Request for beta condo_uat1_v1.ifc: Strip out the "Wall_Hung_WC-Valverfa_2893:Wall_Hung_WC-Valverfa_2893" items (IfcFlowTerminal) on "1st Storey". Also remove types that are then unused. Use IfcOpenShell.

First a look at what the model holds.

```python
import ifcopenshell
import ifcopenshell.util.element

model = ifcopenshell.open("beta condo_uat1_v1.ifc")
print(model.schema)
storey = next(s for s in model.by_type("IfcBuildingStorey") if s.Name == "1st Storey")
terminals = [e for e in ifcopenshell.util.element.get_decomposition(storey) if e.is_a("IfcFlowTerminal")]
seen = {}
for e in terminals:
    element_type = ifcopenshell.util.element.get_type(e)
    name = element_type.Name if element_type not in (None, e) else None
    seen[name] = seen.get(name, 0) + 1
for name, count in sorted(seen.items(), key=str):
    print(count, "x", name)
```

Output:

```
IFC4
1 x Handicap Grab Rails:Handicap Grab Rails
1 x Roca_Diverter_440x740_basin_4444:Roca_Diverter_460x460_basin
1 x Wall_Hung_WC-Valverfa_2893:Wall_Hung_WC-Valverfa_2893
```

```python
import ifcopenshell
import ifcopenshell.api.root
import ifcopenshell.util.element

model = ifcopenshell.open("beta condo_uat1_v1.ifc")

storey = next(s for s in model.by_type("IfcBuildingStorey") if s.Name == "1st Storey")
terminals = [e for e in ifcopenshell.util.element.get_decomposition(storey) if e.is_a("IfcFlowTerminal")]
targets = [e for e in terminals if (t := ifcopenshell.util.element.get_type(e)) not in (None, e) and t.Name == "Wall_Hung_WC-Valverfa_2893:Wall_Hung_WC-Valverfa_2893"]
types = {ifcopenshell.util.element.get_type(e) for e in targets} - {None, *targets}

for e in targets:
    ifcopenshell.api.root.remove_product(model, product=e)
print(len(targets), "removed")

unused = [t for t in types if not ifcopenshell.util.element.get_types(t)]
for t in unused:
    ifcopenshell.api.root.remove_product(model, product=t)
print(len(unused), "unused types removed")

model.write("beta condo_uat1_v1_rev.ifc")
```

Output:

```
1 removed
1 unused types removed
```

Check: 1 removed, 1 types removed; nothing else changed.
